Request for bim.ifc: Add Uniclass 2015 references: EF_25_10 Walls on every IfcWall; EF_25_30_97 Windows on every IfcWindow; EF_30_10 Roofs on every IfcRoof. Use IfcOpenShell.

First a look at what the model holds.

```python
import ifcopenshell

model = ifcopenshell.open("bim.ifc")
print(model.schema)
print("classifications:", [c.Name for c in model.by_type("IfcClassification")])
for ifc_class in ("IfcDoor", "IfcRoof", "IfcStair", "IfcWall", "IfcWindow"):
    print(ifc_class, len(model.by_type(ifc_class)))
```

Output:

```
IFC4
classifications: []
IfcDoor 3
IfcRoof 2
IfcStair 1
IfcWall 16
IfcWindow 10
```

```python
import ifcopenshell
import ifcopenshell.api.classification

model = ifcopenshell.open("bim.ifc")

system = ifcopenshell.api.classification.add_classification(model, classification="Uniclass 2015")

codes = {
    "IfcWall": ("EF_25_10", "Walls"),
    "IfcWindow": ("EF_25_30_97", "Windows"),
    "IfcRoof": ("EF_30_10", "Roofs"),
}
for ifc_class, (code, name) in codes.items():
    products = model.by_type(ifc_class)
    ifcopenshell.api.classification.add_reference(
        model, products=products, classification=system, identification=code, name=name
    )
    print(code, len(products))

model.write("bim_v2.ifc")
```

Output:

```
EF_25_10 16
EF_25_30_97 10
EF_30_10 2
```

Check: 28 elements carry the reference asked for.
